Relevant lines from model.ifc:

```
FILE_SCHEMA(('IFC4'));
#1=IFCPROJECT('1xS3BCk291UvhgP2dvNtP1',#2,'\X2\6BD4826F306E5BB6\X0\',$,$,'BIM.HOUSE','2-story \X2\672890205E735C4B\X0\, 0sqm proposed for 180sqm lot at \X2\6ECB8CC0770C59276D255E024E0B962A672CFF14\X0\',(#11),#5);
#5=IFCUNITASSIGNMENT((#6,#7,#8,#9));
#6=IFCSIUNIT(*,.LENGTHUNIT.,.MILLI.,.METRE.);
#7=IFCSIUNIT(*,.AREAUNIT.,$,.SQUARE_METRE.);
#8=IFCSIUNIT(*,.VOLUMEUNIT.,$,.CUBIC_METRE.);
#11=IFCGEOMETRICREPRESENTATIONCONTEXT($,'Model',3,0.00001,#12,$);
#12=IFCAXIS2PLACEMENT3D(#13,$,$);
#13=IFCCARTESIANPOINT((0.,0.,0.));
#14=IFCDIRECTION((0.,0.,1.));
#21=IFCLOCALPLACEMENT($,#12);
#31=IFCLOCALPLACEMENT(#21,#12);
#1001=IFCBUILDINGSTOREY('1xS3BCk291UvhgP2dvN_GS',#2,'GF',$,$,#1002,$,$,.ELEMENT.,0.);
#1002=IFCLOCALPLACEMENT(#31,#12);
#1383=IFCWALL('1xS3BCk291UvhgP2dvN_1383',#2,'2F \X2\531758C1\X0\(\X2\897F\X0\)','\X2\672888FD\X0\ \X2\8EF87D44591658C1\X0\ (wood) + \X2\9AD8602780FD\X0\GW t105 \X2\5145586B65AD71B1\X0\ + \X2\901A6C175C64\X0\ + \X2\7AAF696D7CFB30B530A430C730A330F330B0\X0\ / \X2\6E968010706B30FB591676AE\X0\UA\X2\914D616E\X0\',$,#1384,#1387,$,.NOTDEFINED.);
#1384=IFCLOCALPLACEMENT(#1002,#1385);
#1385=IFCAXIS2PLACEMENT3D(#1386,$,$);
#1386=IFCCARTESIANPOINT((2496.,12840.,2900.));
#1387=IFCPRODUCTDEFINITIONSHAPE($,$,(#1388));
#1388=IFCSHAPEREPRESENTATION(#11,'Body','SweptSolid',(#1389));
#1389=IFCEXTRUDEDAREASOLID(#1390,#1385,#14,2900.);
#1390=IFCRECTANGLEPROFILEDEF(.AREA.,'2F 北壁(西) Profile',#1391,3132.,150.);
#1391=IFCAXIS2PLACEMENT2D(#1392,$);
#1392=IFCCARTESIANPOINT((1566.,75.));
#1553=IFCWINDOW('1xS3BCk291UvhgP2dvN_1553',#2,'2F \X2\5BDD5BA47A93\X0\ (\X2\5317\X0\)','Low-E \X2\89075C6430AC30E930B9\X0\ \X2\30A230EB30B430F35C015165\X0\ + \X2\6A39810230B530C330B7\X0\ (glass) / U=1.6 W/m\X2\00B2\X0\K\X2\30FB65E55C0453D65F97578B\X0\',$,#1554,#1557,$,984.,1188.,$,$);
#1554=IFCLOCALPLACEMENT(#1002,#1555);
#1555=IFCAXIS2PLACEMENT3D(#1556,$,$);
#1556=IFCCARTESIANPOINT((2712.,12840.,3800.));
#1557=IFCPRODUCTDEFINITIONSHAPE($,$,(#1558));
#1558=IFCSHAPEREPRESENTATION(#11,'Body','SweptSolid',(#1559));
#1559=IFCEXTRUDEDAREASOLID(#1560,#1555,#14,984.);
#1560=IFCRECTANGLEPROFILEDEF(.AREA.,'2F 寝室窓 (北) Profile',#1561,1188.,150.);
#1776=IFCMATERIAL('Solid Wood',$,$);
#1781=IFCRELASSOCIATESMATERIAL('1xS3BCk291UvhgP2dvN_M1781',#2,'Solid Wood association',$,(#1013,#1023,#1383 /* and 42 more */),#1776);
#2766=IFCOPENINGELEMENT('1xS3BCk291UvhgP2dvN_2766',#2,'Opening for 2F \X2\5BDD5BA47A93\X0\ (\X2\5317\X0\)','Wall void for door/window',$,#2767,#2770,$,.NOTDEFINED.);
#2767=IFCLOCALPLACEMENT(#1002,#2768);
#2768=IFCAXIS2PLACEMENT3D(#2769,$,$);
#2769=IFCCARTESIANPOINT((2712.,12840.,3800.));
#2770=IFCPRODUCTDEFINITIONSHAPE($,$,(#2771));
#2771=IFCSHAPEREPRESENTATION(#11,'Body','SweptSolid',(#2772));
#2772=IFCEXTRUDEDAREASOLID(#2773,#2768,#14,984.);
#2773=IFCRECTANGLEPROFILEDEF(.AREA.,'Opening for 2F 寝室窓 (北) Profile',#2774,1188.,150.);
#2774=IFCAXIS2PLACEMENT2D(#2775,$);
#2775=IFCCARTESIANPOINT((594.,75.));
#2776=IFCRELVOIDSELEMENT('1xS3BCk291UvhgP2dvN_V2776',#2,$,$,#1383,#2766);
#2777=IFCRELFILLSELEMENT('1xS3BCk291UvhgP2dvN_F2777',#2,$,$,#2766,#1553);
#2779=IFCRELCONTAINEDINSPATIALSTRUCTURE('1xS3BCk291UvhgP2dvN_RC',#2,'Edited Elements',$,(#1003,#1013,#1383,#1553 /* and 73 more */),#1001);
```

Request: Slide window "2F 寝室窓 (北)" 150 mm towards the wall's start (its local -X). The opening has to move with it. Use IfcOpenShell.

```python
import ifcopenshell
import ifcopenshell.api.geometry
import ifcopenshell.util.placement
import ifcopenshell.util.unit

model = ifcopenshell.open("model.ifc")
unit_scale = ifcopenshell.util.unit.calculate_unit_scale(model)

window = model.by_guid("1xS3BCk291UvhgP2dvN_1553")
opening = window.FillsVoids[0].RelatingOpeningElement
wall = opening.VoidsElements[0].RelatingBuildingElement

wall_matrix = ifcopenshell.util.placement.get_local_placement(wall.ObjectPlacement)
shift = wall_matrix[:3, 0] * -0.15 / unit_scale
before = ifcopenshell.util.placement.get_local_placement(window.ObjectPlacement)[:3, 3].copy()

# The window is not placed relative to its opening, so move both.
for product in (opening, window):
    matrix = ifcopenshell.util.placement.get_local_placement(product.ObjectPlacement)
    matrix[:3, 3] += shift
    ifcopenshell.api.geometry.edit_object_placement(model, product=product, matrix=matrix, is_si=False)

after = ifcopenshell.util.placement.get_local_placement(window.ObjectPlacement)[:3, 3]
print("window moved by", (after - before).round(3) + 0.0)

model.write("model_v2.ifc")
```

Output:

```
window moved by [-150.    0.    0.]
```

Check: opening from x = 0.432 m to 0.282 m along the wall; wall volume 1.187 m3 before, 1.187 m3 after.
